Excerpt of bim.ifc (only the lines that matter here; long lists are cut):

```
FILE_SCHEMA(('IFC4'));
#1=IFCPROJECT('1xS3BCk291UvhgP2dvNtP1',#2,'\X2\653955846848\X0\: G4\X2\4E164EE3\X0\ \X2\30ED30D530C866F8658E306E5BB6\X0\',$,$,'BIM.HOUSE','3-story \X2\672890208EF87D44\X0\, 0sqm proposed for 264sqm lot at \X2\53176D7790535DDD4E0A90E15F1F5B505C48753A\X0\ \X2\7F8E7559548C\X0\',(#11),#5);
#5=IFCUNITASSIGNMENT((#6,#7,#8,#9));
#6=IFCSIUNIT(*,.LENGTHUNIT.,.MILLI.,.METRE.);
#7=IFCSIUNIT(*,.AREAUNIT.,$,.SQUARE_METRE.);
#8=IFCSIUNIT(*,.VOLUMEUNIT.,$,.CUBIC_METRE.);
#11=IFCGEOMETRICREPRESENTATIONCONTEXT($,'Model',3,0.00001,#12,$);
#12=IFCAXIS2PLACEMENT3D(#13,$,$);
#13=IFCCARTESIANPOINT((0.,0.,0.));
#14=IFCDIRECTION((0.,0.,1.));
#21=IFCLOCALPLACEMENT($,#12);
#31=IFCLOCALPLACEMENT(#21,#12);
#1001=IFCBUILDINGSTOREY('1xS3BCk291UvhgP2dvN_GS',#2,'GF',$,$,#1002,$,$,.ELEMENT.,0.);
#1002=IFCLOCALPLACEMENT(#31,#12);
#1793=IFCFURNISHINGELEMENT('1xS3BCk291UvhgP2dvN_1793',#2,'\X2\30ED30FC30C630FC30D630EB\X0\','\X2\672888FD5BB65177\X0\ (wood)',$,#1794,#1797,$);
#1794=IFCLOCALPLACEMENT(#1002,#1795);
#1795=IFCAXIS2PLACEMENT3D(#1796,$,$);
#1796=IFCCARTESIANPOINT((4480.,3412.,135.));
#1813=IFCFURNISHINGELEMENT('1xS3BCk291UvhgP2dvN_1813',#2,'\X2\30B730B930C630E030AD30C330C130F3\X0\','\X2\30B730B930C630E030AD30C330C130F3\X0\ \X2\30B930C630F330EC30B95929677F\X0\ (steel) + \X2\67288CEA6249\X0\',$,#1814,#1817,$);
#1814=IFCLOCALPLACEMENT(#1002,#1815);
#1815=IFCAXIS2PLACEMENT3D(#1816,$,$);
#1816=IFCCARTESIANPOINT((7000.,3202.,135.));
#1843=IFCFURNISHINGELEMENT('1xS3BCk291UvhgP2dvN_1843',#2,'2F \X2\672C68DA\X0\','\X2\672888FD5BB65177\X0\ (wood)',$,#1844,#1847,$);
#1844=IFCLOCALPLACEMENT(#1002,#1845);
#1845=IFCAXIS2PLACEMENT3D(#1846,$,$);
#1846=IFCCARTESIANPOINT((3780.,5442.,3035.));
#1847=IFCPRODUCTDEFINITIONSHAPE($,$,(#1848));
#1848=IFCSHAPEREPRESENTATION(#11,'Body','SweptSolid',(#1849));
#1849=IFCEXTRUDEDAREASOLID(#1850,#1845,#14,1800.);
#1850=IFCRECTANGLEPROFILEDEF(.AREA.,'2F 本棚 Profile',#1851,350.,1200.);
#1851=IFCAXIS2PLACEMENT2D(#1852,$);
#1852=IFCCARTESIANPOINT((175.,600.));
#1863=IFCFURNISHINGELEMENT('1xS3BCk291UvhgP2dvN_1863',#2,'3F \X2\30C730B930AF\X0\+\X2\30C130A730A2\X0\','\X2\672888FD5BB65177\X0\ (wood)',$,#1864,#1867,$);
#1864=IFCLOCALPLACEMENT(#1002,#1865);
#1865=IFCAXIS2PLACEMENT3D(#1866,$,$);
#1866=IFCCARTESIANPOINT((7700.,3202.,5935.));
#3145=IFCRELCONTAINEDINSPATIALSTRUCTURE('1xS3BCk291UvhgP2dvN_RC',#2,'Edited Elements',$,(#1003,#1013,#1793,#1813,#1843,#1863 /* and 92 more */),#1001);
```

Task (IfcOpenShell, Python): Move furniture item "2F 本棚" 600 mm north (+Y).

```python
import ifcopenshell
import ifcopenshell.api.geometry
import ifcopenshell.util.placement
import ifcopenshell.util.unit

model = ifcopenshell.open("bim.ifc")
unit_scale = ifcopenshell.util.unit.calculate_unit_scale(model)

item = model.by_guid("1xS3BCk291UvhgP2dvN_1843")
matrix = ifcopenshell.util.placement.get_local_placement(item.ObjectPlacement)
matrix[1, 3] += 0.6 / unit_scale
ifcopenshell.api.geometry.edit_object_placement(model, product=item, matrix=matrix, is_si=False)

print(ifcopenshell.util.placement.get_local_placement(item.ObjectPlacement).round(3) + 0.0)

model.write("bim_edited.ifc")
```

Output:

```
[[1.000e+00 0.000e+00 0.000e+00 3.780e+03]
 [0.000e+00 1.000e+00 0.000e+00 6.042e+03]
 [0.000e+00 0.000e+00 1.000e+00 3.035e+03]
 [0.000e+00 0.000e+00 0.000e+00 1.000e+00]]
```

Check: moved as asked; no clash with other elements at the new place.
